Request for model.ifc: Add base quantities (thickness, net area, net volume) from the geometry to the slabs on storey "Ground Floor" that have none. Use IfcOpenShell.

First a look at what the model holds.

```python
import ifcopenshell
import ifcopenshell.util.element
import ifcopenshell.util.unit

model = ifcopenshell.open("model.ifc")
print(model.schema)
for unit_type in ("LENGTHUNIT", "AREAUNIT", "VOLUMEUNIT"):
    print(unit_type, ifcopenshell.util.unit.calculate_unit_scale(model, unit_type))
storey = next(s for s in model.by_type("IfcBuildingStorey") if s.Name == "Ground Floor")
slabs = [e for e in ifcopenshell.util.element.get_decomposition(storey) if e.is_a("IfcSlab")]
for e in sorted(slabs, key=lambda e: e.id()):
    print(e.id(), e.is_a(), e.Name, list(ifcopenshell.util.element.get_psets(e, qtos_only=True)), sep=" | ")
```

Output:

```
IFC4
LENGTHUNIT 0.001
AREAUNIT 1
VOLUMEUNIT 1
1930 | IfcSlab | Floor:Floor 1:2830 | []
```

```python
import ifcopenshell
import ifcopenshell.api.pset
import ifcopenshell.geom
import ifcopenshell.util.element
import ifcopenshell.util.shape
import ifcopenshell.util.unit

model = ifcopenshell.open("model.ifc")
unit_scale = ifcopenshell.util.unit.calculate_unit_scale(model)
area_scale = ifcopenshell.util.unit.calculate_unit_scale(model, "AREAUNIT")
volume_scale = ifcopenshell.util.unit.calculate_unit_scale(model, "VOLUMEUNIT")
settings = ifcopenshell.geom.settings()

storey = next(s for s in model.by_type("IfcBuildingStorey") if s.Name == "Ground Floor")
slabs = [e for e in ifcopenshell.util.element.get_decomposition(storey) if e.is_a("IfcSlab")]

for e in sorted(slabs, key=lambda e: e.id()):
    if ifcopenshell.util.element.get_psets(e, qtos_only=True, should_inherit=False):
        continue
    # Geometry comes back in metres, in the element's own axes.
    shape = ifcopenshell.geom.create_shape(settings, e)
    values = {
        "Width": ifcopenshell.util.shape.get_z(shape.geometry) / unit_scale,
        "NetArea": ifcopenshell.util.shape.get_footprint_area(shape.geometry) / area_scale,
        "NetVolume": ifcopenshell.util.shape.get_volume(shape.geometry) / volume_scale,
    }
    qto = ifcopenshell.api.pset.add_qto(model, product=e, name="Qto_SlabBaseQuantities")
    ifcopenshell.api.pset.edit_qto(model, qto=qto, properties=values)
    print(e.id(), {k: round(v, 3) for k, v in values.items()})

model.write("model-out.ifc")
```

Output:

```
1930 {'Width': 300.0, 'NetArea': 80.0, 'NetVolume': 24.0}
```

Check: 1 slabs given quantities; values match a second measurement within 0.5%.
